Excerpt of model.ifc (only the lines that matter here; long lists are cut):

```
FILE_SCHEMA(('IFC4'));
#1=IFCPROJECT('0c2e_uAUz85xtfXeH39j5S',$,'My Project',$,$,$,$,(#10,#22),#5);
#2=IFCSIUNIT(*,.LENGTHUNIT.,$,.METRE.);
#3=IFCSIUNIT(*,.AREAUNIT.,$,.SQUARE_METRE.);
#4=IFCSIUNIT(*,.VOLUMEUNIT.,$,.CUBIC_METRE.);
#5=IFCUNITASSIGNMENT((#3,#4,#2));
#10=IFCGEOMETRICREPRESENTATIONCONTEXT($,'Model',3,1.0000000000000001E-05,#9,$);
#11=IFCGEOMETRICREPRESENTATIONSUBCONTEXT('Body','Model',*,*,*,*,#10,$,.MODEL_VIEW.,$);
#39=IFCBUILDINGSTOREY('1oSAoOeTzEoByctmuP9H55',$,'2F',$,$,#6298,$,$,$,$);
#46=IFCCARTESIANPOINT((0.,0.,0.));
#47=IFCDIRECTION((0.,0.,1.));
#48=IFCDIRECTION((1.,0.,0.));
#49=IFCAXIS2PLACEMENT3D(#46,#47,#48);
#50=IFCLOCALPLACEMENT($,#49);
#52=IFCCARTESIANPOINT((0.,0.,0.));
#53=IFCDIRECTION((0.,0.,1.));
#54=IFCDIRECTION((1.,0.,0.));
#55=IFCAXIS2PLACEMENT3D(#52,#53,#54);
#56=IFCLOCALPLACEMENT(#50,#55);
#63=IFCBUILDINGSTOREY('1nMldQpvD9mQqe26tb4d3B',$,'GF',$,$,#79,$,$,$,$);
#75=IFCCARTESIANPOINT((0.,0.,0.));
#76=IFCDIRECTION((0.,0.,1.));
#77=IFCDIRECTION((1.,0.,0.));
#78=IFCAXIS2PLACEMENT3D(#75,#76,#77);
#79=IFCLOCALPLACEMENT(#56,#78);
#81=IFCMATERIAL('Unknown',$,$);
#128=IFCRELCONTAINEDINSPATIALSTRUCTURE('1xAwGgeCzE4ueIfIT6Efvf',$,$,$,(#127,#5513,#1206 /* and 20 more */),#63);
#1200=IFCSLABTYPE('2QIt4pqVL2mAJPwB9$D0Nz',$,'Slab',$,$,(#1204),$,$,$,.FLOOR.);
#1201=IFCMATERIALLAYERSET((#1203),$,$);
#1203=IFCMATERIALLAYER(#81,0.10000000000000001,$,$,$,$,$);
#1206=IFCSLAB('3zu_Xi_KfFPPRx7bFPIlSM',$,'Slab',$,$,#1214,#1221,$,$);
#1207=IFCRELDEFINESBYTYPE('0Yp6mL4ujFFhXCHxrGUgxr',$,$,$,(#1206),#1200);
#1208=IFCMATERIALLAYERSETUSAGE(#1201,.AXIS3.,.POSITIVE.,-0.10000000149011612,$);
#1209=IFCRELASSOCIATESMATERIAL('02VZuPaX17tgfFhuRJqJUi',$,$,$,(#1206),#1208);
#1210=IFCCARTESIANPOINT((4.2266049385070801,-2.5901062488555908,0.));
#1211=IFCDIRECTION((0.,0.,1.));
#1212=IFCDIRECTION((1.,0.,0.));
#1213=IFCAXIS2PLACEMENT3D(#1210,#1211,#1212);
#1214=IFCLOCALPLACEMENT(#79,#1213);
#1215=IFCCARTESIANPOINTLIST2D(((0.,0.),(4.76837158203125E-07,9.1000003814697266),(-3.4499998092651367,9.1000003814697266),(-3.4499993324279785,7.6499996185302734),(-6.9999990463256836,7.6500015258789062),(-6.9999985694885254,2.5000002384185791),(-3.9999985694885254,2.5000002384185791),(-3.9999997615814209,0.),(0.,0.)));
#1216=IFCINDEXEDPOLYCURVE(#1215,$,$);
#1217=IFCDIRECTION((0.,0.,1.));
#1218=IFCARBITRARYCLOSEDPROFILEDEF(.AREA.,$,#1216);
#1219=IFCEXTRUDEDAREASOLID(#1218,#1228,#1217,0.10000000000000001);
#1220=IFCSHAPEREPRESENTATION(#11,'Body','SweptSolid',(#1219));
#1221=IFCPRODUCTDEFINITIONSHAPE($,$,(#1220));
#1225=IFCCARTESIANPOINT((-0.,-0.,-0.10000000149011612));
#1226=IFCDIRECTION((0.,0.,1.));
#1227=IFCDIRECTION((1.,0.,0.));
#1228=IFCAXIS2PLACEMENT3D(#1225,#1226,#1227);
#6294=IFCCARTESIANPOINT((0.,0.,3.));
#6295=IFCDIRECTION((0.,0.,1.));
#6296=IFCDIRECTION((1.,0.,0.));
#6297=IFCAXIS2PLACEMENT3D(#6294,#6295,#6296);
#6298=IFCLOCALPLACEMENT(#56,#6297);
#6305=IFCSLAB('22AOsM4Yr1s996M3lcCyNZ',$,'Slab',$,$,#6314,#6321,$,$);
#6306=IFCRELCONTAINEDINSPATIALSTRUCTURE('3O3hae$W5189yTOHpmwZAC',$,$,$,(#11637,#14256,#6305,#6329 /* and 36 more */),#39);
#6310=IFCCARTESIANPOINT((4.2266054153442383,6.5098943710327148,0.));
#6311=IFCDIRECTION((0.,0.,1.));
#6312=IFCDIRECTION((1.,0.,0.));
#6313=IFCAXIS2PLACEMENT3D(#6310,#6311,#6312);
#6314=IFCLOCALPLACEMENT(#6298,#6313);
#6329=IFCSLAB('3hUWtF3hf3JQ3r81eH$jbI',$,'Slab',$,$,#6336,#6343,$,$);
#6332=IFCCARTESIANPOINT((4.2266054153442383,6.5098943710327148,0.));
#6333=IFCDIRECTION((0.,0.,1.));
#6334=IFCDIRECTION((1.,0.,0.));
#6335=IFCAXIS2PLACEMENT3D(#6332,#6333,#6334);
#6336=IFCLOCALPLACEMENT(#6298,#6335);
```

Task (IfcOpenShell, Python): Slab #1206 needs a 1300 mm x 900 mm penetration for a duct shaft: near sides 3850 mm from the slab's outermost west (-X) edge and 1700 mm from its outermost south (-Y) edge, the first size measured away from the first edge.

```python
import numpy as np
import ifcopenshell
import ifcopenshell.api.feature
import ifcopenshell.api.geometry
import ifcopenshell.api.root
import ifcopenshell.geom
import ifcopenshell.util.placement
import ifcopenshell.util.representation
import ifcopenshell.util.shape
import ifcopenshell.util.unit

model = ifcopenshell.open("model.ifc")
unit_scale = ifcopenshell.util.unit.calculate_unit_scale(model)
settings = ifcopenshell.geom.settings()


def volume(element):
    """Net volume in cubic metres, openings subtracted."""
    shape = ifcopenshell.geom.create_shape(settings, element)
    return ifcopenshell.util.shape.get_volume(shape.geometry)


slab = model.by_guid("3zu_Xi_KfFPPRx7bFPIlSM")
before = volume(slab)

# Extent in the slab's own axes, in metres. The edges named are its -X and -Y sides.
slab_shape = ifcopenshell.geom.create_shape(settings, slab)
vertices = ifcopenshell.util.shape.get_vertices(slab_shape.geometry)
x_min, y_min, bottom = vertices.min(axis=0)
top = vertices[:, 2].max()

opening = ifcopenshell.api.root.create_entity(model, ifc_class="IfcOpeningElement", name="Duct shaft opening", predefined_type="OPENING")
context = ifcopenshell.util.representation.get_context(model, "Model", "Body", "MODEL_VIEW")
width, depth = 1.3, 0.9
outline = [(0.0, 0.0), (width, 0.0), (width, depth), (0.0, depth), (0.0, 0.0)]
# Overshoot both faces by 50 mm so the cut is clean.
shape = ifcopenshell.api.geometry.add_slab_representation(
    model, context=context, depth=top - bottom + 0.1, polyline=outline
)
ifcopenshell.api.geometry.assign_representation(model, product=opening, representation=shape)

matrix = ifcopenshell.util.placement.get_local_placement(slab.ObjectPlacement)
matrix[:, 3] = matrix @ np.append(np.array([x_min + 3.85, y_min + 1.7, bottom - 0.05]) / unit_scale, 1.0)
ifcopenshell.api.geometry.edit_object_placement(model, product=opening, matrix=matrix, is_si=False)
ifcopenshell.api.feature.add_feature(model, feature=opening, element=slab)

after = volume(slab)

print(f"slab volume {before:.3f} -> {after:.3f} m3")

model.write("model_edited.ifc")
```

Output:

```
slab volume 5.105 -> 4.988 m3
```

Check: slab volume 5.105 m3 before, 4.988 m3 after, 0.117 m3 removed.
